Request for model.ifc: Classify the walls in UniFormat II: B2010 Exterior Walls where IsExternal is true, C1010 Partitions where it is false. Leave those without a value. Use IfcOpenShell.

First a look at what the model holds.

```python
import ifcopenshell
import ifcopenshell.util.element

model = ifcopenshell.open("model.ifc")
print(model.schema)
print("classifications:", [c.Name for c in model.by_type("IfcClassification")])
values = [ifcopenshell.util.element.get_pset(e, "Pset_WallCommon", "IsExternal") for e in model.by_type("IfcWall")]
for value in (True, False, None):
    print("IsExternal", value, values.count(value))
```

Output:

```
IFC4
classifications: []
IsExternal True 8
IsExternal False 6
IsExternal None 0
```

```python
import ifcopenshell
import ifcopenshell.api.classification
import ifcopenshell.util.element

model = ifcopenshell.open("model.ifc")

system = ifcopenshell.api.classification.add_classification(model, classification="UniFormat II")

walls = model.by_type("IfcWall")
external = {e: ifcopenshell.util.element.get_pset(e, "Pset_WallCommon", "IsExternal") for e in walls}
for flag, code, name in ((True, "B2010", "Exterior Walls"), (False, "C1010", "Partitions")):
    products = [e for e in walls if external[e] is flag]
    ifcopenshell.api.classification.add_reference(
        model, products=products, classification=system, identification=code, name=name
    )
    print(code, len(products))

model.write("model_v2.ifc")
```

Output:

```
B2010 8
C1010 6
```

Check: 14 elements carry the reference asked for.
